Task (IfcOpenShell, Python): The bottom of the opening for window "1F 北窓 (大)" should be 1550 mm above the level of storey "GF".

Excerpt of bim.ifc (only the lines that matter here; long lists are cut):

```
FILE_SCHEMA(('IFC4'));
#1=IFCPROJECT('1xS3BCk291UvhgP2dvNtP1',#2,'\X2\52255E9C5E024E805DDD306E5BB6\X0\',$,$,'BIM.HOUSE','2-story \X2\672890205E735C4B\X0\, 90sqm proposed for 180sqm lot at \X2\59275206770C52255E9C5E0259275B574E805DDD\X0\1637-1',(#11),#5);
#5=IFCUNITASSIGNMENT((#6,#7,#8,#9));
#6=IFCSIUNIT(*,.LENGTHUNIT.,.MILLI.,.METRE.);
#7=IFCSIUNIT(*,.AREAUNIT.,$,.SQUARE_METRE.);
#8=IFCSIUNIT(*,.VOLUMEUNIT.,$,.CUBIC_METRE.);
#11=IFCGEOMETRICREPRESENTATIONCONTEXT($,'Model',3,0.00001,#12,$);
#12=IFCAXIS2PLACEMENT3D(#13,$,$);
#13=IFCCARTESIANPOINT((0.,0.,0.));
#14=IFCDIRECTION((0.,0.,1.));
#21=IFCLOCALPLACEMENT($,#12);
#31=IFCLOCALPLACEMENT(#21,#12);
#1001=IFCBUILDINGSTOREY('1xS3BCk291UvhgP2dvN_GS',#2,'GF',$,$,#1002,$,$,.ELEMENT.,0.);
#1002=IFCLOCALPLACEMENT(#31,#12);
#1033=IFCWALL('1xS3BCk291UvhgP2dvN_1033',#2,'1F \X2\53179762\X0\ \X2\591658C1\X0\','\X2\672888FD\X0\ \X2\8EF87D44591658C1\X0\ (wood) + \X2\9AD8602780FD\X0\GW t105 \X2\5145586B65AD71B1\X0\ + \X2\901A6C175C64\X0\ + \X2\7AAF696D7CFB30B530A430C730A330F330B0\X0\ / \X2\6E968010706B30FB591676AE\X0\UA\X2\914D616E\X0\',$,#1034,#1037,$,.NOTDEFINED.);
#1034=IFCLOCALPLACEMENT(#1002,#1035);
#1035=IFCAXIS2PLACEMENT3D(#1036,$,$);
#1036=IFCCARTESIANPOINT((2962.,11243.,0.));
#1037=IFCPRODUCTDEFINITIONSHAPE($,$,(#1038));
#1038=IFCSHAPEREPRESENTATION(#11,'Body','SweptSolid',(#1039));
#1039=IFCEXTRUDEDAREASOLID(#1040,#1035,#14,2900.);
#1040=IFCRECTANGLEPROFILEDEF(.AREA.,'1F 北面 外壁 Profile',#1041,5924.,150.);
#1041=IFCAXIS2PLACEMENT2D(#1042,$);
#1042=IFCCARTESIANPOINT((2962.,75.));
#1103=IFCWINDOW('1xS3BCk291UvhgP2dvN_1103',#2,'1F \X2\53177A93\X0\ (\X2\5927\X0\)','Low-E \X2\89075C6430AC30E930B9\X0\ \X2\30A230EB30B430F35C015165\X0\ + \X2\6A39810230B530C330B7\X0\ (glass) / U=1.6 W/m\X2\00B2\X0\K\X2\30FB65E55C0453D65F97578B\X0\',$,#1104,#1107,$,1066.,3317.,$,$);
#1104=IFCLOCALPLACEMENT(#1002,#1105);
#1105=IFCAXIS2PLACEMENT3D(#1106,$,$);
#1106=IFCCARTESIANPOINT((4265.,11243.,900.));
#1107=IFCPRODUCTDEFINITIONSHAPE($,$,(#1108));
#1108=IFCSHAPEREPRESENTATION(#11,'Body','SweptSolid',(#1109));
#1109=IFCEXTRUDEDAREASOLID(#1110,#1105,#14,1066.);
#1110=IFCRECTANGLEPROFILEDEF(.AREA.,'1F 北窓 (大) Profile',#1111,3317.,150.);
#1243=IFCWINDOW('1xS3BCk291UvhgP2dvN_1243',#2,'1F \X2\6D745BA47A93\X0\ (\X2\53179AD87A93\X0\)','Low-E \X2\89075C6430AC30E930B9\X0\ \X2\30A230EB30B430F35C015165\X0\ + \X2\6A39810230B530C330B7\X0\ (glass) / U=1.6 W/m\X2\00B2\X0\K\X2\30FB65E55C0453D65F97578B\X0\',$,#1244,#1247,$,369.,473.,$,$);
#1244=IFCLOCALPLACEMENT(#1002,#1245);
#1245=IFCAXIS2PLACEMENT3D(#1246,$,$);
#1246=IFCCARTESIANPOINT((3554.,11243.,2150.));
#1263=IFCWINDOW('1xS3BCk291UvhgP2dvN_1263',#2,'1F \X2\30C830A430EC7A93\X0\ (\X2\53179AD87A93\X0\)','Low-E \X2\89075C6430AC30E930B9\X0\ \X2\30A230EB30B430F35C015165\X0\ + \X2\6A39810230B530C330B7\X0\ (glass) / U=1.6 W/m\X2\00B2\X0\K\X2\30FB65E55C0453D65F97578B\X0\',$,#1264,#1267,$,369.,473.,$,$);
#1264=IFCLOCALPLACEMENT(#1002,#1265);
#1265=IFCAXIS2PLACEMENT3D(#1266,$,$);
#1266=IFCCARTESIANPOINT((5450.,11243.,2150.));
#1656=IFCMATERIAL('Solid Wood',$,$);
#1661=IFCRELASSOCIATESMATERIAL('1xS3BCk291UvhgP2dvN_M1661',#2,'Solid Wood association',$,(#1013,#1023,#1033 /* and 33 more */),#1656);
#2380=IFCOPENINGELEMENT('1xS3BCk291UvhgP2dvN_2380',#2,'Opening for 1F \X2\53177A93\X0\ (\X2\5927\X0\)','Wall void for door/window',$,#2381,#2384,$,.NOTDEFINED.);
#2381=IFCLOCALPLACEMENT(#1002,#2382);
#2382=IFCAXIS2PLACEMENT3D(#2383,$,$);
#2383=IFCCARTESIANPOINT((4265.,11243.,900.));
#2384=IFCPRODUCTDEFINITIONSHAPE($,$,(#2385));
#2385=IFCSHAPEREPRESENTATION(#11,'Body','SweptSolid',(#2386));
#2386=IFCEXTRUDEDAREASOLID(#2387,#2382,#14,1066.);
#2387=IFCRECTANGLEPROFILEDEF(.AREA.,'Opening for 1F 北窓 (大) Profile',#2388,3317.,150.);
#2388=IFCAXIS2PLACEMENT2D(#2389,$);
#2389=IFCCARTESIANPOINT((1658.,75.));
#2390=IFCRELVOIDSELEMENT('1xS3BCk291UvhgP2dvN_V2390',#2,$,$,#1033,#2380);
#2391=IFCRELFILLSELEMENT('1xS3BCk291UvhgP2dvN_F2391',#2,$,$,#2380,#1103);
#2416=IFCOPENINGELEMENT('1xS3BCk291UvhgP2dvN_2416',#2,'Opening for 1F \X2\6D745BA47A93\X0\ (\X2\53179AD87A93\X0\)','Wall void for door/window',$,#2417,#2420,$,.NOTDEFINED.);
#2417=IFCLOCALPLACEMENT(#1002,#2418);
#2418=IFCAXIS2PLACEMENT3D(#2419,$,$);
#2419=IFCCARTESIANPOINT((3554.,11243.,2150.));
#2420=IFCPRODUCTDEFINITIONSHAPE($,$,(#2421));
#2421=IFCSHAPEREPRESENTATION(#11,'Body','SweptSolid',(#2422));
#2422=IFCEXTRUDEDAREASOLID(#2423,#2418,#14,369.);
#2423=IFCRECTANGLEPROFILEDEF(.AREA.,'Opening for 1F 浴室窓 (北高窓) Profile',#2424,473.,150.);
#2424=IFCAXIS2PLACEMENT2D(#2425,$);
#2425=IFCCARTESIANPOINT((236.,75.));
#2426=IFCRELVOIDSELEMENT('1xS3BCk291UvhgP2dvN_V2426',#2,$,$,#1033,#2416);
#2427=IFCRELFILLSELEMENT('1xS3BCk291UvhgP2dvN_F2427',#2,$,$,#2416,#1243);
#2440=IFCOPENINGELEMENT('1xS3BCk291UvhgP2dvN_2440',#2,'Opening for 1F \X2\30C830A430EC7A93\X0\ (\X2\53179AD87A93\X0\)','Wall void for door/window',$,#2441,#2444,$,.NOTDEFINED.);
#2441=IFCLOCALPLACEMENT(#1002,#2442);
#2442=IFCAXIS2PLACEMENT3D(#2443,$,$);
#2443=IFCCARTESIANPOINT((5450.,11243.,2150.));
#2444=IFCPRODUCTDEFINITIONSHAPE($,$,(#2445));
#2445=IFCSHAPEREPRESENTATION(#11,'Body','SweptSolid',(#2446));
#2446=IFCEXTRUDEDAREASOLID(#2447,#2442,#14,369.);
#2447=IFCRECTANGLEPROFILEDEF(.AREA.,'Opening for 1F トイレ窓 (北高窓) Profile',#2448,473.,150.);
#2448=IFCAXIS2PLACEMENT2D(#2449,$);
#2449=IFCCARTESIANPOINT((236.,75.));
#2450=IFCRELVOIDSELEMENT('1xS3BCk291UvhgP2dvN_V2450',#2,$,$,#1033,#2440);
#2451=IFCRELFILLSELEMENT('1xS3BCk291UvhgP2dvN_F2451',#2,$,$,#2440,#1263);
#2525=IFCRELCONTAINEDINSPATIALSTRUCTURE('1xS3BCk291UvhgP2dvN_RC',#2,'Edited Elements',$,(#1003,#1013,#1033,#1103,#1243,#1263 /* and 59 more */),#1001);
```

```python
import numpy as np
import ifcopenshell
import ifcopenshell.api.geometry
import ifcopenshell.geom
import ifcopenshell.util.element
import ifcopenshell.util.placement
import ifcopenshell.util.shape
import ifcopenshell.util.unit

model = ifcopenshell.open("bim.ifc")
unit_scale = ifcopenshell.util.unit.calculate_unit_scale(model)

window = model.by_guid("1xS3BCk291UvhgP2dvN_1103")
opening = window.FillsVoids[0].RelatingOpeningElement
storey = ifcopenshell.util.element.get_container(window, ifc_class="IfcBuildingStorey")
level = ifcopenshell.util.placement.get_local_placement(storey.ObjectPlacement)[2, 3]

# The opening's origin need not be at the sill, so measure its lowest point.
shape = ifcopenshell.geom.create_shape(ifcopenshell.geom.settings(), opening)
bottom = ifcopenshell.util.shape.get_shape_bottom_elevation(shape, shape.geometry) / unit_scale
dz = level + 1.55 / unit_scale - bottom

shift = np.array([0.0, 0.0, dz])
# The window is not placed relative to its opening, so move both.
for product in (opening, window):
    matrix = ifcopenshell.util.placement.get_local_placement(product.ObjectPlacement)
    matrix[:3, 3] += shift
    ifcopenshell.api.geometry.edit_object_placement(model, product=product, matrix=matrix, is_si=False)

print(f"moved by {dz * unit_scale:+.3f} m")

model.write("bim_edited.ifc")
```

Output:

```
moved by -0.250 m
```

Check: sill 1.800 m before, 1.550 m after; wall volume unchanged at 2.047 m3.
